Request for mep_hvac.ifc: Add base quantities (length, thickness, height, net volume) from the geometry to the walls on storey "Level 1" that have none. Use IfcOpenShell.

First a look at what the model holds.

```python
import ifcopenshell
import ifcopenshell.util.element
import ifcopenshell.util.unit

model = ifcopenshell.open("mep_hvac.ifc")
print(model.schema)
for unit_type in ("LENGTHUNIT", "AREAUNIT", "VOLUMEUNIT"):
    print(unit_type, ifcopenshell.util.unit.calculate_unit_scale(model, unit_type))
storey = next(s for s in model.by_type("IfcBuildingStorey") if s.Name == "Level 1")
walls = [e for e in ifcopenshell.util.element.get_decomposition(storey) if e.is_a("IfcWall")]
for e in sorted(walls, key=lambda e: e.id()):
    print(e.id(), e.is_a(), e.Name, list(ifcopenshell.util.element.get_psets(e, qtos_only=True)), sep=" | ")
```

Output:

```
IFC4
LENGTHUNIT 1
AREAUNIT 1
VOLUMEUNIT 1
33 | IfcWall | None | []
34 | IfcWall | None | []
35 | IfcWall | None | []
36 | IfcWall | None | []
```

```python
import ifcopenshell
import ifcopenshell.api.pset
import ifcopenshell.geom
import ifcopenshell.util.element
import ifcopenshell.util.shape
import ifcopenshell.util.unit

model = ifcopenshell.open("mep_hvac.ifc")
unit_scale = ifcopenshell.util.unit.calculate_unit_scale(model)
volume_scale = ifcopenshell.util.unit.calculate_unit_scale(model, "VOLUMEUNIT")
settings = ifcopenshell.geom.settings()

storey = next(s for s in model.by_type("IfcBuildingStorey") if s.Name == "Level 1")
walls = [e for e in ifcopenshell.util.element.get_decomposition(storey) if e.is_a("IfcWall")]

for e in sorted(walls, key=lambda e: e.id()):
    if ifcopenshell.util.element.get_psets(e, qtos_only=True, should_inherit=False):
        continue
    # Geometry comes back in metres, in the element's own axes.
    shape = ifcopenshell.geom.create_shape(settings, e)
    values = {
        "Length": ifcopenshell.util.shape.get_x(shape.geometry) / unit_scale,
        "Width": ifcopenshell.util.shape.get_y(shape.geometry) / unit_scale,
        "Height": ifcopenshell.util.shape.get_z(shape.geometry) / unit_scale,
        "NetVolume": ifcopenshell.util.shape.get_volume(shape.geometry) / volume_scale,
    }
    qto = ifcopenshell.api.pset.add_qto(model, product=e, name="Qto_WallBaseQuantities")
    ifcopenshell.api.pset.edit_qto(model, qto=qto, properties=values)
    print(e.id(), {k: round(v, 3) for k, v in values.items()})

model.write("mep_hvac-out.ifc")
```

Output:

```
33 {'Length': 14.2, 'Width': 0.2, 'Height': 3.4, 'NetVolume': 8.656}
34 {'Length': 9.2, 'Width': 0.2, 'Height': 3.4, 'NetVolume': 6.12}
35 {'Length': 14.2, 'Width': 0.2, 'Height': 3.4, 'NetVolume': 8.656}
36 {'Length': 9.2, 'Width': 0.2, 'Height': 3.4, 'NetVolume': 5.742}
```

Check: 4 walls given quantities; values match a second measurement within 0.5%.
